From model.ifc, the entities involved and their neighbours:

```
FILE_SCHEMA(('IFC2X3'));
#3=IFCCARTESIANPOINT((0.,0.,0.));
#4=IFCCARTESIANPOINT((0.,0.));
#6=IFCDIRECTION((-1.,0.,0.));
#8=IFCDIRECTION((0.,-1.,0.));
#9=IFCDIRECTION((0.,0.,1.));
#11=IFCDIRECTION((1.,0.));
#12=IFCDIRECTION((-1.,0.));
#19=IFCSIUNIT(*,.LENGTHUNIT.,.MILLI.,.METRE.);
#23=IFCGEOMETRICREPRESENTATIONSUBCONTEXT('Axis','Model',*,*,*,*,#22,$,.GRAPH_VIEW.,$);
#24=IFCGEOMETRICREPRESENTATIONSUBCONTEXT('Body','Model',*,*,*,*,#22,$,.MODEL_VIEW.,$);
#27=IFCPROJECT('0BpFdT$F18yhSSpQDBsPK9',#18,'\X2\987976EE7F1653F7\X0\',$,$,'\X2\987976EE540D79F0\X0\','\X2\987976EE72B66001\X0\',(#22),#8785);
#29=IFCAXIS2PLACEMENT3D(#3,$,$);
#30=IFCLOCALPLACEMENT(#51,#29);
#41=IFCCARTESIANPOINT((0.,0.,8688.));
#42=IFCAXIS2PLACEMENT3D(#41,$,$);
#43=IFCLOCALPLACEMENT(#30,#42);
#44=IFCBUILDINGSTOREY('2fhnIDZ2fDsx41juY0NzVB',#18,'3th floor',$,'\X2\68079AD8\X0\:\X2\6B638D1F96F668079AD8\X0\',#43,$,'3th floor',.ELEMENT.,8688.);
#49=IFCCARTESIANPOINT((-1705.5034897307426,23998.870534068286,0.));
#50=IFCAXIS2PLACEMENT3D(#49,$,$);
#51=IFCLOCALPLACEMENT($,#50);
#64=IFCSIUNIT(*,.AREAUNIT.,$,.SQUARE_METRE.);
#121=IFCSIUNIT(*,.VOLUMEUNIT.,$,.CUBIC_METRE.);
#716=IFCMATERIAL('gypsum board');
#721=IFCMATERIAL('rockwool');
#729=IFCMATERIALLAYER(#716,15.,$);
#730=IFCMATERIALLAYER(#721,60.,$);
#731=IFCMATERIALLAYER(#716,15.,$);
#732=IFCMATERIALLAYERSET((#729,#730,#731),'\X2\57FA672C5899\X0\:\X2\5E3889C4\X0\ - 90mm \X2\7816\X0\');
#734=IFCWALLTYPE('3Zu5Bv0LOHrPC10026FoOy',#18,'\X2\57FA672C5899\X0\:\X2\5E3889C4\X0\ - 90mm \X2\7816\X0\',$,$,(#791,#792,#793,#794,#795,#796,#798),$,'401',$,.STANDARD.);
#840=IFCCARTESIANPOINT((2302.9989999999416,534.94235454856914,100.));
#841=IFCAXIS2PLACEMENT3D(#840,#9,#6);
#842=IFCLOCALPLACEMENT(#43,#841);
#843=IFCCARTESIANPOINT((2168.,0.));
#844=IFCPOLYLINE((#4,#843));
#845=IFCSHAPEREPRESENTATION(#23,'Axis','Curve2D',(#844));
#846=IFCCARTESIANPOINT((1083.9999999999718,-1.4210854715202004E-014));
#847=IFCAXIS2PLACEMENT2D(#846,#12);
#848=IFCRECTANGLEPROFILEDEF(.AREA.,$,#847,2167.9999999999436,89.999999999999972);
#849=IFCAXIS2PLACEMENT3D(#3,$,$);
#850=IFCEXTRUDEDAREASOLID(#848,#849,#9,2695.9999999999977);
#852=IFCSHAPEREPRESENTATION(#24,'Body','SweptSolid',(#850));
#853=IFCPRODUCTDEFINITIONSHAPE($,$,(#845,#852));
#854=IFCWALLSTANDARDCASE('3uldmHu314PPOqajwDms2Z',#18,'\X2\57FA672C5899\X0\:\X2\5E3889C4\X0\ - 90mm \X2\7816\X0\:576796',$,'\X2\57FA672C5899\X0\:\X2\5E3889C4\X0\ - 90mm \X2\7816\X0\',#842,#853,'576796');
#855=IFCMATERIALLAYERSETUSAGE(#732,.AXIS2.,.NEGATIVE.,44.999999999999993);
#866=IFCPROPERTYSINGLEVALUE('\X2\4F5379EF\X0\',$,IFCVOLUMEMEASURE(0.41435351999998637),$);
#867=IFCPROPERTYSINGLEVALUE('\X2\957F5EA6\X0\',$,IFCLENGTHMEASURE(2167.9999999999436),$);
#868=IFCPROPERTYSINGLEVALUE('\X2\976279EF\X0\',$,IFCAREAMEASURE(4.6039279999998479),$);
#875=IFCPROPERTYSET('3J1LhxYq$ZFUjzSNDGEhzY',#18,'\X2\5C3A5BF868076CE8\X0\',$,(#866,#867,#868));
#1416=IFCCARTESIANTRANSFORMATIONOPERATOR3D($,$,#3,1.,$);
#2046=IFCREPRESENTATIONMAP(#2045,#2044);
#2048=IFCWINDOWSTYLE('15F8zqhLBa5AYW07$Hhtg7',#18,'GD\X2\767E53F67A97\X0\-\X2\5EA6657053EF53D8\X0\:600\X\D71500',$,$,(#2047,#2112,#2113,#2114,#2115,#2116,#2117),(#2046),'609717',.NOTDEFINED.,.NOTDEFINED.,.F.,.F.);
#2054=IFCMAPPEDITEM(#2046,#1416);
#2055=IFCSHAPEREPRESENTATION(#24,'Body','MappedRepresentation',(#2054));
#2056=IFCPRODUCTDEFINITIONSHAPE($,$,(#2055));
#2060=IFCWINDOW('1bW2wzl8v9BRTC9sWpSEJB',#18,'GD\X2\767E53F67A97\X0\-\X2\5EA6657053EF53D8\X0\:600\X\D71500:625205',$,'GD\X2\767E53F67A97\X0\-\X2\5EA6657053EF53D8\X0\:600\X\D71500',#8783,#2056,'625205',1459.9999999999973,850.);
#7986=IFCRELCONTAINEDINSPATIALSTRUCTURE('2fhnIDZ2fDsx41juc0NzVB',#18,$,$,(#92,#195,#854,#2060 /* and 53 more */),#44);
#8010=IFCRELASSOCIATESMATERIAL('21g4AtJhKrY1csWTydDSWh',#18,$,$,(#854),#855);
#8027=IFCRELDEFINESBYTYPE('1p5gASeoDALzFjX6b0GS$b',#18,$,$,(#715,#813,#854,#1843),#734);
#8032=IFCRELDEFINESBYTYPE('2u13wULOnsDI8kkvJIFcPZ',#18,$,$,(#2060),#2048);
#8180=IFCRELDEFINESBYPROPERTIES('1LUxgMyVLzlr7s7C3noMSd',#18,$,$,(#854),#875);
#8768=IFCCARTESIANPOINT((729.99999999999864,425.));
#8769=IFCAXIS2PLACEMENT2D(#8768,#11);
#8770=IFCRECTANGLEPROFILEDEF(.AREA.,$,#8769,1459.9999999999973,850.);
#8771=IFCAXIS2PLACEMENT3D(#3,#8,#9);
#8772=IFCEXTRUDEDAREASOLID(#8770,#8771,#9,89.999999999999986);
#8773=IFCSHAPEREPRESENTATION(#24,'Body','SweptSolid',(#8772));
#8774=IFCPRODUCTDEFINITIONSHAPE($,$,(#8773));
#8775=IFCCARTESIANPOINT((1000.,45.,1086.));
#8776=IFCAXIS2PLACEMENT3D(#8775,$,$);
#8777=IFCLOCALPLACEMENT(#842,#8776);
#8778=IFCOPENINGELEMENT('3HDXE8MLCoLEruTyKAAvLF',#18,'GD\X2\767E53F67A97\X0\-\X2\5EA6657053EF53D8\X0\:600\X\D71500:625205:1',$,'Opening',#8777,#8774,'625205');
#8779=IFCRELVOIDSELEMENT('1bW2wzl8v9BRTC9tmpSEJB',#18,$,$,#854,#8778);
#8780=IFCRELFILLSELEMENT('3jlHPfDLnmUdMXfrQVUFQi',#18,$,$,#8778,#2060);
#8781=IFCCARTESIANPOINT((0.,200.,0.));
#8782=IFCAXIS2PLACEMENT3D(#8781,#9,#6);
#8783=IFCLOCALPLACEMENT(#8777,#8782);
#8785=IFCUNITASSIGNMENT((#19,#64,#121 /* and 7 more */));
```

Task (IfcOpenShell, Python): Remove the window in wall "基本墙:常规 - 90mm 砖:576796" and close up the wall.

```python
import ifcopenshell
import ifcopenshell.api.feature
import ifcopenshell.api.pset
import ifcopenshell.api.root
import ifcopenshell.geom
import ifcopenshell.util.element
import ifcopenshell.util.shape
import ifcopenshell.util.unit

model = ifcopenshell.open("model.ifc")
area_scale = ifcopenshell.util.unit.calculate_unit_scale(model, "AREAUNIT")
volume_scale = ifcopenshell.util.unit.calculate_unit_scale(model, "VOLUMEUNIT")
settings = ifcopenshell.geom.settings()


def volume(element):
    """Net volume in cubic metres, openings subtracted."""
    shape = ifcopenshell.geom.create_shape(settings, element)
    return ifcopenshell.util.shape.get_volume(shape.geometry)


window = model.by_id(2060)
opening = window.FillsVoids[0].RelatingOpeningElement
wall = opening.VoidsElements[0].RelatingBuildingElement
before = volume(wall)

ifcopenshell.api.root.remove_product(model, product=window)
ifcopenshell.api.feature.remove_feature(model, feature=opening)

after = volume(wall)
thickness = 0.09  # wall thickness in metres

# Update the wall's stored quantities.
pset = model.by_id(ifcopenshell.util.element.get_pset(wall, "尺寸标注", should_inherit=False)["id"])
ifcopenshell.api.pset.edit_pset(model, pset=pset, properties={
    "体积": model.create_entity("IfcVolumeMeasure", after / volume_scale),
    "面积": model.create_entity("IfcAreaMeasure", after / thickness / area_scale),
})

print(f"wall volume {before:.3f} -> {after:.3f} m3")

model.write("model_updated.ifc")
```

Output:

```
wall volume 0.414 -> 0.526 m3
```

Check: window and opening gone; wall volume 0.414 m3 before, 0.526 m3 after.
